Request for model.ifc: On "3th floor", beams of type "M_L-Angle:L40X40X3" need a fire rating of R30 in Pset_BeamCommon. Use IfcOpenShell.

First a look at what the model holds.

```python
import ifcopenshell
import ifcopenshell.util.element

model = ifcopenshell.open("model.ifc")
print(model.schema)
storey = next(s for s in model.by_type("IfcBuildingStorey") if s.Name == "3th floor")
beams = [e for e in ifcopenshell.util.element.get_decomposition(storey) if e.is_a("IfcBeam")]
seen = {}
for e in beams:
    element_type = ifcopenshell.util.element.get_type(e)
    key = (element_type.Name if element_type != e and element_type else None, ifcopenshell.util.element.get_pset(e, "Pset_BeamCommon", "FireRating"))
    seen[key] = seen.get(key, 0) + 1
for (name, value), count in sorted(seen.items(), key=str):
    print(count, "x", name, "|", value)
```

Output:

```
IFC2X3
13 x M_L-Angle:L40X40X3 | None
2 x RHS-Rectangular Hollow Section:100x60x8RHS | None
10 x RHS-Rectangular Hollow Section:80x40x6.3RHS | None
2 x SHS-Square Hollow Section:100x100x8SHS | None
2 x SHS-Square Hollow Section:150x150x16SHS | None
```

```python
import ifcopenshell
import ifcopenshell.api.pset
import ifcopenshell.util.element

model = ifcopenshell.open("model.ifc")

storey = next(s for s in model.by_type("IfcBuildingStorey") if s.Name == "3th floor")
beams = [e for e in ifcopenshell.util.element.get_decomposition(storey) if e.is_a("IfcBeam")]

count = 0
for e in beams:
    element_type = ifcopenshell.util.element.get_type(e)
    if element_type in (None, e) or element_type.Name != "M_L-Angle:L40X40X3":
        continue
    # add_pset returns the element's existing set when there is one.
    pset = ifcopenshell.api.pset.add_pset(model, product=e, name="Pset_BeamCommon")
    ifcopenshell.api.pset.edit_pset(model, pset=pset, properties={"FireRating": "R30"})
    count += 1

print(count, "beams updated")

model.write("model_updated.ifc")
```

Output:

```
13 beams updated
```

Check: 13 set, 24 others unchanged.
